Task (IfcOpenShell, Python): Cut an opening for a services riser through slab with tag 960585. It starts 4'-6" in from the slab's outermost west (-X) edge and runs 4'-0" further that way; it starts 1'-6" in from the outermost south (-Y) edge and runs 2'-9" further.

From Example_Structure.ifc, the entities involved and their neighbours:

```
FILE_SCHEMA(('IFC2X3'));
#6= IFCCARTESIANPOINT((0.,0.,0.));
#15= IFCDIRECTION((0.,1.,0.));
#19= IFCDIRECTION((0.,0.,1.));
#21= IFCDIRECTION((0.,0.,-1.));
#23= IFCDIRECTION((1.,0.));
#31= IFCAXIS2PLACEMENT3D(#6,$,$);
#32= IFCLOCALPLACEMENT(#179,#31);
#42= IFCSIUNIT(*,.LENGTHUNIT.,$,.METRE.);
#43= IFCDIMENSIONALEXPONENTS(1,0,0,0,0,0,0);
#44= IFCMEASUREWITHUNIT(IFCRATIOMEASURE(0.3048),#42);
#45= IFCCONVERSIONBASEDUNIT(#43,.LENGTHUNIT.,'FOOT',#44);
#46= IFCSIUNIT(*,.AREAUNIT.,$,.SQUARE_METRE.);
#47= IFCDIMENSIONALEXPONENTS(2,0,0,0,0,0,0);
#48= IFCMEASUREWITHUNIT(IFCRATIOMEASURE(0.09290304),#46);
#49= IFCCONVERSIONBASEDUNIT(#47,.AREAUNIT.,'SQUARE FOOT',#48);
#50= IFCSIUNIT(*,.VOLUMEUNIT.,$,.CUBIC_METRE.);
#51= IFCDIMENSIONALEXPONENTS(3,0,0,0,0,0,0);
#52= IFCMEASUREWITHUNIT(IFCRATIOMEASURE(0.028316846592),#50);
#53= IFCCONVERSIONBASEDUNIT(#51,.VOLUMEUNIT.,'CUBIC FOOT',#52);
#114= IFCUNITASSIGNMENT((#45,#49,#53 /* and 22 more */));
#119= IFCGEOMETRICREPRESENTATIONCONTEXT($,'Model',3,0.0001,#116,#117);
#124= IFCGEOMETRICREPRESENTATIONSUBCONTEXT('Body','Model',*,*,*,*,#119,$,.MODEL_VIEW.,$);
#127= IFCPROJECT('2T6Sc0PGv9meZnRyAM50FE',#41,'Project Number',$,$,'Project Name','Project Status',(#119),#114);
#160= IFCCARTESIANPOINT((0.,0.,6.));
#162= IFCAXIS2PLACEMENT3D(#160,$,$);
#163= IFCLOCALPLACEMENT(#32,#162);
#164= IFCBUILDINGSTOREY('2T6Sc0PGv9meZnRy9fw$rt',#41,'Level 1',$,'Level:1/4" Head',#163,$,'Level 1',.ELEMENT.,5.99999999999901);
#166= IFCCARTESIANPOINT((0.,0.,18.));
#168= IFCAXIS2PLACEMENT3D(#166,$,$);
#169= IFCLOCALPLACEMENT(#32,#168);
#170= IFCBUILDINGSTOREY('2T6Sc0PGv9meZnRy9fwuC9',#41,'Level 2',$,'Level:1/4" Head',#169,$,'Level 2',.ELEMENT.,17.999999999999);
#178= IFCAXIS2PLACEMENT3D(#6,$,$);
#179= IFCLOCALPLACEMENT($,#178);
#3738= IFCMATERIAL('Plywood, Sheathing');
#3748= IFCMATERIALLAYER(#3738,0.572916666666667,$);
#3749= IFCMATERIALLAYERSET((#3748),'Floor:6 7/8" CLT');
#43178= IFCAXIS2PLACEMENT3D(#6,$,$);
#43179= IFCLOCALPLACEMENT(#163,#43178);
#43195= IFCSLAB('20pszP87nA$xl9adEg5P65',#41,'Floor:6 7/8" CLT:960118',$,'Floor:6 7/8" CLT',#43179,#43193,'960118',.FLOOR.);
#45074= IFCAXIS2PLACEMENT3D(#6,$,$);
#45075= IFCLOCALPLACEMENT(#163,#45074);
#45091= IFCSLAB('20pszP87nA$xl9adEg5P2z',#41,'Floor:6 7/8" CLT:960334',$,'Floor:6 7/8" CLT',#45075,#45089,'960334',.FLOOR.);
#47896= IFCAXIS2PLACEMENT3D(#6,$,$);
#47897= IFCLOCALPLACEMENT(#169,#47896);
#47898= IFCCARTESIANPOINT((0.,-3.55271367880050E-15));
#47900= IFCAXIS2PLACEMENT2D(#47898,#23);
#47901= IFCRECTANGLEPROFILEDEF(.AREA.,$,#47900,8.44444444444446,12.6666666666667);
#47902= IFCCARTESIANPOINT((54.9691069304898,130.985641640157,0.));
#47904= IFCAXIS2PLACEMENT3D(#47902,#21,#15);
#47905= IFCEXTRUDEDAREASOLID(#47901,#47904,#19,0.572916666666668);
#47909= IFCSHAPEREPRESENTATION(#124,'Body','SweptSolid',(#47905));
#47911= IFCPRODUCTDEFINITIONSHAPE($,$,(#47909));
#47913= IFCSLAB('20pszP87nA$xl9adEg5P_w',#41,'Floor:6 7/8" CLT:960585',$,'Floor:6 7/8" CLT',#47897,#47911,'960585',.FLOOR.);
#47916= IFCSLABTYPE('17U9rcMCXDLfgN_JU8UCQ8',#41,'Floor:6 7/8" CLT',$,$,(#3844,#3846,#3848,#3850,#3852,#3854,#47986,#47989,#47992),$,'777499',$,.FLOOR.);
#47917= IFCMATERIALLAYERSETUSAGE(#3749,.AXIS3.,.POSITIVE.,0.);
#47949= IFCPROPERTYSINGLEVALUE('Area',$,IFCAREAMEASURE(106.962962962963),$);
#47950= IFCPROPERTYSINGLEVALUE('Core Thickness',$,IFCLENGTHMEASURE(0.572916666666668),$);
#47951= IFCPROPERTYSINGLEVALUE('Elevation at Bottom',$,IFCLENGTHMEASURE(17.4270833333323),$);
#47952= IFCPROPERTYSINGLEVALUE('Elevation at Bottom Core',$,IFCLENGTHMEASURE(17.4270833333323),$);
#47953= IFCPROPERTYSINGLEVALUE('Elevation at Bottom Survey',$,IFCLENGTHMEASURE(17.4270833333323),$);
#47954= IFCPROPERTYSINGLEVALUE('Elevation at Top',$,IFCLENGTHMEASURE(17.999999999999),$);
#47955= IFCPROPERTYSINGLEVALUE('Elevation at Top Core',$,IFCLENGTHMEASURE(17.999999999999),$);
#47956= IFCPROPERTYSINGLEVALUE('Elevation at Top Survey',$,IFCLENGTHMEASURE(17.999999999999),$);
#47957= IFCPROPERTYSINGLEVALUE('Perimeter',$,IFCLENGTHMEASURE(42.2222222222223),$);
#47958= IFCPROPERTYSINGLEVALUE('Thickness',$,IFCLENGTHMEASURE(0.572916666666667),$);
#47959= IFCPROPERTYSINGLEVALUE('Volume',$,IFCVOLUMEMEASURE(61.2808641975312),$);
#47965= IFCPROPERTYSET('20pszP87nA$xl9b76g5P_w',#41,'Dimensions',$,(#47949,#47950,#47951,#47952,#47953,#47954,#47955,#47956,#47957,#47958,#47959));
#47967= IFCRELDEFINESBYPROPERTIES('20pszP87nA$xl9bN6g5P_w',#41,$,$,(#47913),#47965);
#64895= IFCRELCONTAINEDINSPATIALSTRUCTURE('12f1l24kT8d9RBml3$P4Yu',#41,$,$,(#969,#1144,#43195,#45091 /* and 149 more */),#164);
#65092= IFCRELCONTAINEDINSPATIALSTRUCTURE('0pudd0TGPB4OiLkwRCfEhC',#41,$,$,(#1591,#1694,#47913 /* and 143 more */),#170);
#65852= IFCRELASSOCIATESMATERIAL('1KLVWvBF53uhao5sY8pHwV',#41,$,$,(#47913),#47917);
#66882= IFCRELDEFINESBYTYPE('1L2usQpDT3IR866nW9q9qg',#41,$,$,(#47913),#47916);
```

```python
import numpy as np
import ifcopenshell
import ifcopenshell.api.feature
import ifcopenshell.api.geometry
import ifcopenshell.api.pset
import ifcopenshell.api.root
import ifcopenshell.geom
import ifcopenshell.util.element
import ifcopenshell.util.placement
import ifcopenshell.util.representation
import ifcopenshell.util.shape
import ifcopenshell.util.unit

model = ifcopenshell.open("Example_Structure.ifc")
unit_scale = ifcopenshell.util.unit.calculate_unit_scale(model)
area_scale = ifcopenshell.util.unit.calculate_unit_scale(model, "AREAUNIT")
volume_scale = ifcopenshell.util.unit.calculate_unit_scale(model, "VOLUMEUNIT")
settings = ifcopenshell.geom.settings()


def volume(element):
    """Net volume in cubic metres, openings subtracted."""
    shape = ifcopenshell.geom.create_shape(settings, element)
    return ifcopenshell.util.shape.get_volume(shape.geometry)


slab = model.by_guid("20pszP87nA$xl9adEg5P_w")
before = volume(slab)

# Extent in the slab's own axes, in metres. The edges named are its -X and -Y sides.
slab_shape = ifcopenshell.geom.create_shape(settings, slab)
vertices = ifcopenshell.util.shape.get_vertices(slab_shape.geometry)
x_min, y_min, bottom = vertices.min(axis=0)
top = vertices[:, 2].max()

opening = ifcopenshell.api.root.create_entity(model, ifc_class="IfcOpeningElement", name="Services riser opening")
context = ifcopenshell.util.representation.get_context(model, "Model", "Body", "MODEL_VIEW")
width, depth = 1.2192, 0.8382
outline = [(0.0, 0.0), (width, 0.0), (width, depth), (0.0, depth), (0.0, 0.0)]
# Overshoot both faces by 50 mm so the cut is clean.
shape = ifcopenshell.api.geometry.add_slab_representation(
    model, context=context, depth=top - bottom + 0.1, polyline=outline
)
ifcopenshell.api.geometry.assign_representation(model, product=opening, representation=shape)

matrix = ifcopenshell.util.placement.get_local_placement(slab.ObjectPlacement)
matrix[:, 3] = matrix @ np.append(np.array([x_min + 1.3716, y_min + 0.4572, bottom - 0.05]) / unit_scale, 1.0)
ifcopenshell.api.geometry.edit_object_placement(model, product=opening, matrix=matrix, is_si=False)
ifcopenshell.api.feature.add_feature(model, feature=opening, element=slab)

after = volume(slab)

# Update the slab's stored quantities.
pset = model.by_id(ifcopenshell.util.element.get_pset(slab, "Dimensions", should_inherit=False)["id"])
ifcopenshell.api.pset.edit_pset(model, pset=pset, properties={
    "Area": model.create_entity("IfcAreaMeasure", after / (top - bottom) / area_scale),
    "Volume": model.create_entity("IfcVolumeMeasure", after / volume_scale),
})

print(f"slab volume {before:.3f} -> {after:.3f} m3")

model.write("Example_Structure_edited.ifc")
```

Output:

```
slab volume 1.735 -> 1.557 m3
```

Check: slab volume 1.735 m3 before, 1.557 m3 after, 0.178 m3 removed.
